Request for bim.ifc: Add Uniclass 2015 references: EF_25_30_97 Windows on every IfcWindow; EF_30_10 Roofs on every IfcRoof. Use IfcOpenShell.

First a look at what the model holds.

```python
import ifcopenshell

model = ifcopenshell.open("bim.ifc")
print(model.schema)
print("classifications:", [c.Name for c in model.by_type("IfcClassification")])
for ifc_class in ("IfcDoor", "IfcRoof", "IfcStair", "IfcWall", "IfcWindow"):
    print(ifc_class, len(model.by_type(ifc_class)))
```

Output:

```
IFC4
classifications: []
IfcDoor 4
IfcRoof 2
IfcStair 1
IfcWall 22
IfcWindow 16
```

```python
import ifcopenshell
import ifcopenshell.api.classification

model = ifcopenshell.open("bim.ifc")

system = ifcopenshell.api.classification.add_classification(model, classification="Uniclass 2015")

codes = {
    "IfcWindow": ("EF_25_30_97", "Windows"),
    "IfcRoof": ("EF_30_10", "Roofs"),
}
for ifc_class, (code, name) in codes.items():
    products = model.by_type(ifc_class)
    ifcopenshell.api.classification.add_reference(
        model, products=products, classification=system, identification=code, name=name
    )
    print(code, len(products))

model.write("bim_v2.ifc")
```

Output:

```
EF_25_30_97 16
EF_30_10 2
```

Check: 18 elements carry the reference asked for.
